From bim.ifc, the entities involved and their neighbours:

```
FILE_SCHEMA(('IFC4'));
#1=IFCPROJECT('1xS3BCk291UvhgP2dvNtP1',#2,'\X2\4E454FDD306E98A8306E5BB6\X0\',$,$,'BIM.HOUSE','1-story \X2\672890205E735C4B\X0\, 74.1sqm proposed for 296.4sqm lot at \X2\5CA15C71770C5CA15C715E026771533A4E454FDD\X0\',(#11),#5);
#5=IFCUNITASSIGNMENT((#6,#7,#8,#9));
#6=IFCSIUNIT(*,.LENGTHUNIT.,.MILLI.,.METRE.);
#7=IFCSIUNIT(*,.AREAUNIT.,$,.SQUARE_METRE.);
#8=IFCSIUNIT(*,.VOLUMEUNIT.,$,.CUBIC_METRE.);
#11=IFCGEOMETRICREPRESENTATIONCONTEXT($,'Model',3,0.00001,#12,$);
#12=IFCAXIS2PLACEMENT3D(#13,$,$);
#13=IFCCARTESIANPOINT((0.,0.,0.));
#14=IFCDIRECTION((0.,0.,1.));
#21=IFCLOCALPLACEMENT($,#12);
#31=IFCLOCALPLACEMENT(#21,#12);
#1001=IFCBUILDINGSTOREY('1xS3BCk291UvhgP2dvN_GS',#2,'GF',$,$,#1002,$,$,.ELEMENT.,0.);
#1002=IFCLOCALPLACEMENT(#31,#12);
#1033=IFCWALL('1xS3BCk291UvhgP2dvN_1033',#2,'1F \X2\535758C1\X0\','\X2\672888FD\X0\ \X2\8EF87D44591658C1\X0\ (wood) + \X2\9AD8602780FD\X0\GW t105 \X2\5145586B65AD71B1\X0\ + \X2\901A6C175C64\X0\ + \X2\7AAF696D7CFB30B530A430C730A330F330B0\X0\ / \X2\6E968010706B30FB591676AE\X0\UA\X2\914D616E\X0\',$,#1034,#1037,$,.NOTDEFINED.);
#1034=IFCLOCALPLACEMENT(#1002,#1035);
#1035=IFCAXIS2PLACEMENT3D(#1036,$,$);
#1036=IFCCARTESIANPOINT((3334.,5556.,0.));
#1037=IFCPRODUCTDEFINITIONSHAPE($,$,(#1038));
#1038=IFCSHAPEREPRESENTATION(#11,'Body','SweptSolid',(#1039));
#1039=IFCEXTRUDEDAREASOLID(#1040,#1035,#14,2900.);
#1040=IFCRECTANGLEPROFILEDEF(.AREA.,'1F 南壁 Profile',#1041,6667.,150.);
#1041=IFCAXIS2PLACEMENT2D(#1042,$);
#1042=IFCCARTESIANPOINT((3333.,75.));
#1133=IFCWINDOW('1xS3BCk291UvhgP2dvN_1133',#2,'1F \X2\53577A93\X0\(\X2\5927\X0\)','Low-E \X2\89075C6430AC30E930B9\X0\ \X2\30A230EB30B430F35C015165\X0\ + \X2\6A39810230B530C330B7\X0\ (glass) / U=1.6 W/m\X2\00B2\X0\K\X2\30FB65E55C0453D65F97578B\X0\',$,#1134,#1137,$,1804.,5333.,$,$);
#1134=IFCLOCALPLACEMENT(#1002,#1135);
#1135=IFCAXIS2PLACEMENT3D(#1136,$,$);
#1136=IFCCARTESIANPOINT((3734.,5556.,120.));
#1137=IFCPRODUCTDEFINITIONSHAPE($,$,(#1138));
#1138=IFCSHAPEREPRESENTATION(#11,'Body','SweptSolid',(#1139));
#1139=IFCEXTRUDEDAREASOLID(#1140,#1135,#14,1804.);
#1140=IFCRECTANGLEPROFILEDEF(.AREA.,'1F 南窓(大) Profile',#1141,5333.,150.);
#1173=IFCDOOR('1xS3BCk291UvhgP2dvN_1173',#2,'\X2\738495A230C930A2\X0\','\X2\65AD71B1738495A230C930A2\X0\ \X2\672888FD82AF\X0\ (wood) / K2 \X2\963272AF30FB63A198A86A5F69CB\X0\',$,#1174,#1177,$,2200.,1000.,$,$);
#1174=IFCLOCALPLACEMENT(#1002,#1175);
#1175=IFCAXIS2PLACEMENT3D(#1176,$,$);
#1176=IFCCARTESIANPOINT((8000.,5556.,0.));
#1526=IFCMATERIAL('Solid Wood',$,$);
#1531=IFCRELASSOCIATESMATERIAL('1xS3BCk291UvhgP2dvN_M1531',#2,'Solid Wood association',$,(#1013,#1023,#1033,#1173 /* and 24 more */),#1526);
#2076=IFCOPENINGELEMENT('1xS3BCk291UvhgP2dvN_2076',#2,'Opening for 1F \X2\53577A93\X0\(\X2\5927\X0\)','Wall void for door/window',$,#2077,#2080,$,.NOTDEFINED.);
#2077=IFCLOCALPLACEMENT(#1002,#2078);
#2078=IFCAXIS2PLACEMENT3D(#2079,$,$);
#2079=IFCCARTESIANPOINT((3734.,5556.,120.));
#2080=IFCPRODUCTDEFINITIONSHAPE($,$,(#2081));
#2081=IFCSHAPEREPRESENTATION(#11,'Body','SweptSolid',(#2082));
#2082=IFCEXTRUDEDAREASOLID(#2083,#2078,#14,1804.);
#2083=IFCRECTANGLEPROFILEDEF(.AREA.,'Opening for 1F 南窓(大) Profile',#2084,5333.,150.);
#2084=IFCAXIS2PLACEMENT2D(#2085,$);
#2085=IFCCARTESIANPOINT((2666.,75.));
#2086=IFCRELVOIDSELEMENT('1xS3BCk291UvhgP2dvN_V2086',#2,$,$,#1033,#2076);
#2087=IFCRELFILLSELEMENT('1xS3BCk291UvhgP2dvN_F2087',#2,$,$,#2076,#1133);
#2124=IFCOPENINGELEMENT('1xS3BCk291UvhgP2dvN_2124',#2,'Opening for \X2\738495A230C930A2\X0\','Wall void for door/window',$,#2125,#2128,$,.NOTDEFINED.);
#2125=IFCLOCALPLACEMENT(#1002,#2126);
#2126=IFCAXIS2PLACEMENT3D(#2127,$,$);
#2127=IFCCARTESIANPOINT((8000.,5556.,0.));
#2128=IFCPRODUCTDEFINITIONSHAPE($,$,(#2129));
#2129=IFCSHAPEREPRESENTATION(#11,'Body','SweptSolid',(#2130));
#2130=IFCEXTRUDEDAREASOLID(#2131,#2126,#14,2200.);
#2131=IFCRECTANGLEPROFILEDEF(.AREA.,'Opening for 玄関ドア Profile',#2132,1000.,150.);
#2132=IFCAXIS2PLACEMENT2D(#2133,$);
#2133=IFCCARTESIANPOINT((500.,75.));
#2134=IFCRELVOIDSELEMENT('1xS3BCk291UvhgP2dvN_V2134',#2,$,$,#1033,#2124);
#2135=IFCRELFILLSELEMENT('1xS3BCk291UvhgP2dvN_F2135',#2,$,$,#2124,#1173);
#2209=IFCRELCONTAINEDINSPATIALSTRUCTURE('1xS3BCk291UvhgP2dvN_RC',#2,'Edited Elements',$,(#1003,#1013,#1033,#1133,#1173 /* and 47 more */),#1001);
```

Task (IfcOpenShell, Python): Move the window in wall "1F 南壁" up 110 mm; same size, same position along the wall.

```python
import numpy as np
import ifcopenshell
import ifcopenshell.api.geometry
import ifcopenshell.util.placement
import ifcopenshell.util.unit

model = ifcopenshell.open("bim.ifc")
unit_scale = ifcopenshell.util.unit.calculate_unit_scale(model)

window = model.by_id(1133)
opening = window.FillsVoids[0].RelatingOpeningElement
dz = 0.11 / unit_scale

shift = np.array([0.0, 0.0, dz])
# The window is not placed relative to its opening, so move both.
for product in (opening, window):
    matrix = ifcopenshell.util.placement.get_local_placement(product.ObjectPlacement)
    matrix[:3, 3] += shift
    ifcopenshell.api.geometry.edit_object_placement(model, product=product, matrix=matrix, is_si=False)

print(f"moved by {dz * unit_scale:+.3f} m")

model.write("bim_edited.ifc")
```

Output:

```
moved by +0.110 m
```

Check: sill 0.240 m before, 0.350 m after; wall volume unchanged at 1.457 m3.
